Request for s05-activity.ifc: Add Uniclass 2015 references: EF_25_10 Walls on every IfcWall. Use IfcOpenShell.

First a look at what the model holds.

```python
import ifcopenshell

model = ifcopenshell.open("s05-activity.ifc")
print(model.schema)
print("classifications:", [c.Name for c in model.by_type("IfcClassification")])
for ifc_class in ("IfcDoor", "IfcRoof", "IfcStair", "IfcWall", "IfcWindow"):
    print(ifc_class, len(model.by_type(ifc_class)))
```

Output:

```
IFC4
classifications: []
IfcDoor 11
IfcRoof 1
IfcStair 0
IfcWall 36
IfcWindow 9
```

```python
import ifcopenshell
import ifcopenshell.api.classification

model = ifcopenshell.open("s05-activity.ifc")

system = ifcopenshell.api.classification.add_classification(model, classification="Uniclass 2015")

codes = {
    "IfcWall": ("EF_25_10", "Walls"),
}
for ifc_class, (code, name) in codes.items():
    products = model.by_type(ifc_class)
    ifcopenshell.api.classification.add_reference(
        model, products=products, classification=system, identification=code, name=name
    )
    print(code, len(products))

model.write("s05-activity-out.ifc")
```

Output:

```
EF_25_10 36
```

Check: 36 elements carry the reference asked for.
